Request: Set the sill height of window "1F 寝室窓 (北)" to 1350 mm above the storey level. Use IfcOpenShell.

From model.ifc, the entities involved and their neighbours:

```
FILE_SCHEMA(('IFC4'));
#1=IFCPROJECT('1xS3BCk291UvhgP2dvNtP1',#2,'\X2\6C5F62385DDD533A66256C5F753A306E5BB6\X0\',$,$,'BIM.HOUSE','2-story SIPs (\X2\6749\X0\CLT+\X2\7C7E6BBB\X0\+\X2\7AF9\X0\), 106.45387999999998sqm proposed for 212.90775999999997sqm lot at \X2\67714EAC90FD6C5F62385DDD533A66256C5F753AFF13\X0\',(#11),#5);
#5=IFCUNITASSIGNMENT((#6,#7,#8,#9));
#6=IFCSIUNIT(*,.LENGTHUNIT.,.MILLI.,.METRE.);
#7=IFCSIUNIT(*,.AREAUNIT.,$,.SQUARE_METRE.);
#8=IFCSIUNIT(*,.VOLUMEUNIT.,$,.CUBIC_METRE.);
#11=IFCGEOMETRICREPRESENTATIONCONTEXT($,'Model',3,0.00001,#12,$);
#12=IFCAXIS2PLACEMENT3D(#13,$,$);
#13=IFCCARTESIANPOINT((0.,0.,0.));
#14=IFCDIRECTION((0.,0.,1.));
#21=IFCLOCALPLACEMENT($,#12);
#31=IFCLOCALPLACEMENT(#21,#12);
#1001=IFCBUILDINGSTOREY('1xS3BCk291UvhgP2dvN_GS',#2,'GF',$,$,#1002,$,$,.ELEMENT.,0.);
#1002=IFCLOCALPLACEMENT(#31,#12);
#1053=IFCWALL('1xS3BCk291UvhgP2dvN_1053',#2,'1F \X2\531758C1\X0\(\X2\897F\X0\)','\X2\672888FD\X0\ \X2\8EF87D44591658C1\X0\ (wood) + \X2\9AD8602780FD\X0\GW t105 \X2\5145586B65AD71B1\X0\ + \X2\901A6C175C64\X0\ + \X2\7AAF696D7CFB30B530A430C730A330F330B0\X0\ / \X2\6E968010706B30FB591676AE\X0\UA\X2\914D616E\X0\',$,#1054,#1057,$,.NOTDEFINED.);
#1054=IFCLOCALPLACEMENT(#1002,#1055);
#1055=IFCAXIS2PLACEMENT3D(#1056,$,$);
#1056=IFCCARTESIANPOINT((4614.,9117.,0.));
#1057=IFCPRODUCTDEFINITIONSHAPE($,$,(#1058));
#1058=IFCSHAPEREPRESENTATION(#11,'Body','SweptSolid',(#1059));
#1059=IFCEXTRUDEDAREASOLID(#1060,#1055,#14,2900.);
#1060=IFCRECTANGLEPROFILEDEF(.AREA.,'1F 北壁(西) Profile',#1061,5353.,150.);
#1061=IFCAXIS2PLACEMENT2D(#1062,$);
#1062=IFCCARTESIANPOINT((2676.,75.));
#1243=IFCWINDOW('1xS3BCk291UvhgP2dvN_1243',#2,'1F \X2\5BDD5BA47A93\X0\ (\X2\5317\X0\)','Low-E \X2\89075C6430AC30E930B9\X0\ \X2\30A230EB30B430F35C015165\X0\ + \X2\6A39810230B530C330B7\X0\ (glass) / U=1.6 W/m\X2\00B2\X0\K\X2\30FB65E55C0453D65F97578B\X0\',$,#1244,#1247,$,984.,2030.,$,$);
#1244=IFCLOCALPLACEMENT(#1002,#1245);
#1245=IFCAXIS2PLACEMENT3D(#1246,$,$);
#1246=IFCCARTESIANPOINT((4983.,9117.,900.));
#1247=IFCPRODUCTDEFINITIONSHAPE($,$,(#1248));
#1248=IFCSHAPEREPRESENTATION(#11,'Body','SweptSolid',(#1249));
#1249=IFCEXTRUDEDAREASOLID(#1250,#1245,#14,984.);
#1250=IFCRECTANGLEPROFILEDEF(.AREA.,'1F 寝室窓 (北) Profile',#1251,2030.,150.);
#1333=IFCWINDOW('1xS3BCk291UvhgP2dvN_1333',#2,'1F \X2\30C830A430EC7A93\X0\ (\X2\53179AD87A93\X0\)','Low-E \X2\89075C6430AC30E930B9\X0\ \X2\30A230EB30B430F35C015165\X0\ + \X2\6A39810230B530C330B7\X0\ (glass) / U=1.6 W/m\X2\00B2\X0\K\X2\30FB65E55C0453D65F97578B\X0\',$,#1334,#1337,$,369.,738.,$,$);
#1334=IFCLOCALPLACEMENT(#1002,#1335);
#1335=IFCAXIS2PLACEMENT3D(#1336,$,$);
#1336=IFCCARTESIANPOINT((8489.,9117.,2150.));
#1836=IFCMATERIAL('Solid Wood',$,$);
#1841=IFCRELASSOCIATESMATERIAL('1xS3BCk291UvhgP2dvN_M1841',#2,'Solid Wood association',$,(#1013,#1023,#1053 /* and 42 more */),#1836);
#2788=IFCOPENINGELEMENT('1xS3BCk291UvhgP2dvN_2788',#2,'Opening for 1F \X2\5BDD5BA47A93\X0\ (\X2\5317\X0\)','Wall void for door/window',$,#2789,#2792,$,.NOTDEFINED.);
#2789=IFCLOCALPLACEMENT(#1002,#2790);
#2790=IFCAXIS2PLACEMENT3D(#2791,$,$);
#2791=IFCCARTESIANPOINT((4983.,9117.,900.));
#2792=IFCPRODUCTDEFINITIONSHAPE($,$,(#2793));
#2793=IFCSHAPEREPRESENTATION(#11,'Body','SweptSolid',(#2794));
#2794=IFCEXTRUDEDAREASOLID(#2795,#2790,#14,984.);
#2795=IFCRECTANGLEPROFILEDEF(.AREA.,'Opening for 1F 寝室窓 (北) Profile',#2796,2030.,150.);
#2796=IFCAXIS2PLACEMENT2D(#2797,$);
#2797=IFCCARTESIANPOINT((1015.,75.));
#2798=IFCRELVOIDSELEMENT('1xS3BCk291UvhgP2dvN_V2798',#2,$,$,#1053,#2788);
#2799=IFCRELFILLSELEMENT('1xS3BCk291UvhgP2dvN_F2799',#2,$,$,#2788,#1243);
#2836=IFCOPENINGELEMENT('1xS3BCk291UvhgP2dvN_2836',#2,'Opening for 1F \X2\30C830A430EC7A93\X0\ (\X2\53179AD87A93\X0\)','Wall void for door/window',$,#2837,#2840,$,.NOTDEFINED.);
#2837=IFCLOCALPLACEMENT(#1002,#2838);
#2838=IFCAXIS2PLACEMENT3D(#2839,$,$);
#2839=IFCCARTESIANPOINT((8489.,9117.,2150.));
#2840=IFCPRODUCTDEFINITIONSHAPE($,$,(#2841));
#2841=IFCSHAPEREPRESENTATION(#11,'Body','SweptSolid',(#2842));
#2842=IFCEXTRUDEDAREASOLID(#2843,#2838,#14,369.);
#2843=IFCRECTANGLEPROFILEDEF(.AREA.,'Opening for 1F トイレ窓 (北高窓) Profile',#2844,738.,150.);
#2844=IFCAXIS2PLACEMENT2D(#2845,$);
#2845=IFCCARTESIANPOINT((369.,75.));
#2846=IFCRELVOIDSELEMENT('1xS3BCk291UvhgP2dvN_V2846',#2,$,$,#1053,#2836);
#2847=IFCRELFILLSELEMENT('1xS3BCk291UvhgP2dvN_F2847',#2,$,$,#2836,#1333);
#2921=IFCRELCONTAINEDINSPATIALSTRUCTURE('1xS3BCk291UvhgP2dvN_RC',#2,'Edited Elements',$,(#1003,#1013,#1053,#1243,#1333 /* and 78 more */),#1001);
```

```python
import numpy as np
import ifcopenshell
import ifcopenshell.api.geometry
import ifcopenshell.geom
import ifcopenshell.util.element
import ifcopenshell.util.placement
import ifcopenshell.util.shape
import ifcopenshell.util.unit

model = ifcopenshell.open("model.ifc")
unit_scale = ifcopenshell.util.unit.calculate_unit_scale(model)

window = model.by_guid("1xS3BCk291UvhgP2dvN_1243")
opening = window.FillsVoids[0].RelatingOpeningElement
storey = ifcopenshell.util.element.get_container(window, ifc_class="IfcBuildingStorey")
level = ifcopenshell.util.placement.get_local_placement(storey.ObjectPlacement)[2, 3]

# The opening's origin need not be at the sill, so measure its lowest point.
shape = ifcopenshell.geom.create_shape(ifcopenshell.geom.settings(), opening)
bottom = ifcopenshell.util.shape.get_shape_bottom_elevation(shape, shape.geometry) / unit_scale
dz = level + 1.35 / unit_scale - bottom

shift = np.array([0.0, 0.0, dz])
# The window is not placed relative to its opening, so move both.
for product in (opening, window):
    matrix = ifcopenshell.util.placement.get_local_placement(product.ObjectPlacement)
    matrix[:3, 3] += shift
    ifcopenshell.api.geometry.edit_object_placement(model, product=product, matrix=matrix, is_si=False)

print(f"moved by {dz * unit_scale:+.3f} m")

model.write("model_updated.ifc")
```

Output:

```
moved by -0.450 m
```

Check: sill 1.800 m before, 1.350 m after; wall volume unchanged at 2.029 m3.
